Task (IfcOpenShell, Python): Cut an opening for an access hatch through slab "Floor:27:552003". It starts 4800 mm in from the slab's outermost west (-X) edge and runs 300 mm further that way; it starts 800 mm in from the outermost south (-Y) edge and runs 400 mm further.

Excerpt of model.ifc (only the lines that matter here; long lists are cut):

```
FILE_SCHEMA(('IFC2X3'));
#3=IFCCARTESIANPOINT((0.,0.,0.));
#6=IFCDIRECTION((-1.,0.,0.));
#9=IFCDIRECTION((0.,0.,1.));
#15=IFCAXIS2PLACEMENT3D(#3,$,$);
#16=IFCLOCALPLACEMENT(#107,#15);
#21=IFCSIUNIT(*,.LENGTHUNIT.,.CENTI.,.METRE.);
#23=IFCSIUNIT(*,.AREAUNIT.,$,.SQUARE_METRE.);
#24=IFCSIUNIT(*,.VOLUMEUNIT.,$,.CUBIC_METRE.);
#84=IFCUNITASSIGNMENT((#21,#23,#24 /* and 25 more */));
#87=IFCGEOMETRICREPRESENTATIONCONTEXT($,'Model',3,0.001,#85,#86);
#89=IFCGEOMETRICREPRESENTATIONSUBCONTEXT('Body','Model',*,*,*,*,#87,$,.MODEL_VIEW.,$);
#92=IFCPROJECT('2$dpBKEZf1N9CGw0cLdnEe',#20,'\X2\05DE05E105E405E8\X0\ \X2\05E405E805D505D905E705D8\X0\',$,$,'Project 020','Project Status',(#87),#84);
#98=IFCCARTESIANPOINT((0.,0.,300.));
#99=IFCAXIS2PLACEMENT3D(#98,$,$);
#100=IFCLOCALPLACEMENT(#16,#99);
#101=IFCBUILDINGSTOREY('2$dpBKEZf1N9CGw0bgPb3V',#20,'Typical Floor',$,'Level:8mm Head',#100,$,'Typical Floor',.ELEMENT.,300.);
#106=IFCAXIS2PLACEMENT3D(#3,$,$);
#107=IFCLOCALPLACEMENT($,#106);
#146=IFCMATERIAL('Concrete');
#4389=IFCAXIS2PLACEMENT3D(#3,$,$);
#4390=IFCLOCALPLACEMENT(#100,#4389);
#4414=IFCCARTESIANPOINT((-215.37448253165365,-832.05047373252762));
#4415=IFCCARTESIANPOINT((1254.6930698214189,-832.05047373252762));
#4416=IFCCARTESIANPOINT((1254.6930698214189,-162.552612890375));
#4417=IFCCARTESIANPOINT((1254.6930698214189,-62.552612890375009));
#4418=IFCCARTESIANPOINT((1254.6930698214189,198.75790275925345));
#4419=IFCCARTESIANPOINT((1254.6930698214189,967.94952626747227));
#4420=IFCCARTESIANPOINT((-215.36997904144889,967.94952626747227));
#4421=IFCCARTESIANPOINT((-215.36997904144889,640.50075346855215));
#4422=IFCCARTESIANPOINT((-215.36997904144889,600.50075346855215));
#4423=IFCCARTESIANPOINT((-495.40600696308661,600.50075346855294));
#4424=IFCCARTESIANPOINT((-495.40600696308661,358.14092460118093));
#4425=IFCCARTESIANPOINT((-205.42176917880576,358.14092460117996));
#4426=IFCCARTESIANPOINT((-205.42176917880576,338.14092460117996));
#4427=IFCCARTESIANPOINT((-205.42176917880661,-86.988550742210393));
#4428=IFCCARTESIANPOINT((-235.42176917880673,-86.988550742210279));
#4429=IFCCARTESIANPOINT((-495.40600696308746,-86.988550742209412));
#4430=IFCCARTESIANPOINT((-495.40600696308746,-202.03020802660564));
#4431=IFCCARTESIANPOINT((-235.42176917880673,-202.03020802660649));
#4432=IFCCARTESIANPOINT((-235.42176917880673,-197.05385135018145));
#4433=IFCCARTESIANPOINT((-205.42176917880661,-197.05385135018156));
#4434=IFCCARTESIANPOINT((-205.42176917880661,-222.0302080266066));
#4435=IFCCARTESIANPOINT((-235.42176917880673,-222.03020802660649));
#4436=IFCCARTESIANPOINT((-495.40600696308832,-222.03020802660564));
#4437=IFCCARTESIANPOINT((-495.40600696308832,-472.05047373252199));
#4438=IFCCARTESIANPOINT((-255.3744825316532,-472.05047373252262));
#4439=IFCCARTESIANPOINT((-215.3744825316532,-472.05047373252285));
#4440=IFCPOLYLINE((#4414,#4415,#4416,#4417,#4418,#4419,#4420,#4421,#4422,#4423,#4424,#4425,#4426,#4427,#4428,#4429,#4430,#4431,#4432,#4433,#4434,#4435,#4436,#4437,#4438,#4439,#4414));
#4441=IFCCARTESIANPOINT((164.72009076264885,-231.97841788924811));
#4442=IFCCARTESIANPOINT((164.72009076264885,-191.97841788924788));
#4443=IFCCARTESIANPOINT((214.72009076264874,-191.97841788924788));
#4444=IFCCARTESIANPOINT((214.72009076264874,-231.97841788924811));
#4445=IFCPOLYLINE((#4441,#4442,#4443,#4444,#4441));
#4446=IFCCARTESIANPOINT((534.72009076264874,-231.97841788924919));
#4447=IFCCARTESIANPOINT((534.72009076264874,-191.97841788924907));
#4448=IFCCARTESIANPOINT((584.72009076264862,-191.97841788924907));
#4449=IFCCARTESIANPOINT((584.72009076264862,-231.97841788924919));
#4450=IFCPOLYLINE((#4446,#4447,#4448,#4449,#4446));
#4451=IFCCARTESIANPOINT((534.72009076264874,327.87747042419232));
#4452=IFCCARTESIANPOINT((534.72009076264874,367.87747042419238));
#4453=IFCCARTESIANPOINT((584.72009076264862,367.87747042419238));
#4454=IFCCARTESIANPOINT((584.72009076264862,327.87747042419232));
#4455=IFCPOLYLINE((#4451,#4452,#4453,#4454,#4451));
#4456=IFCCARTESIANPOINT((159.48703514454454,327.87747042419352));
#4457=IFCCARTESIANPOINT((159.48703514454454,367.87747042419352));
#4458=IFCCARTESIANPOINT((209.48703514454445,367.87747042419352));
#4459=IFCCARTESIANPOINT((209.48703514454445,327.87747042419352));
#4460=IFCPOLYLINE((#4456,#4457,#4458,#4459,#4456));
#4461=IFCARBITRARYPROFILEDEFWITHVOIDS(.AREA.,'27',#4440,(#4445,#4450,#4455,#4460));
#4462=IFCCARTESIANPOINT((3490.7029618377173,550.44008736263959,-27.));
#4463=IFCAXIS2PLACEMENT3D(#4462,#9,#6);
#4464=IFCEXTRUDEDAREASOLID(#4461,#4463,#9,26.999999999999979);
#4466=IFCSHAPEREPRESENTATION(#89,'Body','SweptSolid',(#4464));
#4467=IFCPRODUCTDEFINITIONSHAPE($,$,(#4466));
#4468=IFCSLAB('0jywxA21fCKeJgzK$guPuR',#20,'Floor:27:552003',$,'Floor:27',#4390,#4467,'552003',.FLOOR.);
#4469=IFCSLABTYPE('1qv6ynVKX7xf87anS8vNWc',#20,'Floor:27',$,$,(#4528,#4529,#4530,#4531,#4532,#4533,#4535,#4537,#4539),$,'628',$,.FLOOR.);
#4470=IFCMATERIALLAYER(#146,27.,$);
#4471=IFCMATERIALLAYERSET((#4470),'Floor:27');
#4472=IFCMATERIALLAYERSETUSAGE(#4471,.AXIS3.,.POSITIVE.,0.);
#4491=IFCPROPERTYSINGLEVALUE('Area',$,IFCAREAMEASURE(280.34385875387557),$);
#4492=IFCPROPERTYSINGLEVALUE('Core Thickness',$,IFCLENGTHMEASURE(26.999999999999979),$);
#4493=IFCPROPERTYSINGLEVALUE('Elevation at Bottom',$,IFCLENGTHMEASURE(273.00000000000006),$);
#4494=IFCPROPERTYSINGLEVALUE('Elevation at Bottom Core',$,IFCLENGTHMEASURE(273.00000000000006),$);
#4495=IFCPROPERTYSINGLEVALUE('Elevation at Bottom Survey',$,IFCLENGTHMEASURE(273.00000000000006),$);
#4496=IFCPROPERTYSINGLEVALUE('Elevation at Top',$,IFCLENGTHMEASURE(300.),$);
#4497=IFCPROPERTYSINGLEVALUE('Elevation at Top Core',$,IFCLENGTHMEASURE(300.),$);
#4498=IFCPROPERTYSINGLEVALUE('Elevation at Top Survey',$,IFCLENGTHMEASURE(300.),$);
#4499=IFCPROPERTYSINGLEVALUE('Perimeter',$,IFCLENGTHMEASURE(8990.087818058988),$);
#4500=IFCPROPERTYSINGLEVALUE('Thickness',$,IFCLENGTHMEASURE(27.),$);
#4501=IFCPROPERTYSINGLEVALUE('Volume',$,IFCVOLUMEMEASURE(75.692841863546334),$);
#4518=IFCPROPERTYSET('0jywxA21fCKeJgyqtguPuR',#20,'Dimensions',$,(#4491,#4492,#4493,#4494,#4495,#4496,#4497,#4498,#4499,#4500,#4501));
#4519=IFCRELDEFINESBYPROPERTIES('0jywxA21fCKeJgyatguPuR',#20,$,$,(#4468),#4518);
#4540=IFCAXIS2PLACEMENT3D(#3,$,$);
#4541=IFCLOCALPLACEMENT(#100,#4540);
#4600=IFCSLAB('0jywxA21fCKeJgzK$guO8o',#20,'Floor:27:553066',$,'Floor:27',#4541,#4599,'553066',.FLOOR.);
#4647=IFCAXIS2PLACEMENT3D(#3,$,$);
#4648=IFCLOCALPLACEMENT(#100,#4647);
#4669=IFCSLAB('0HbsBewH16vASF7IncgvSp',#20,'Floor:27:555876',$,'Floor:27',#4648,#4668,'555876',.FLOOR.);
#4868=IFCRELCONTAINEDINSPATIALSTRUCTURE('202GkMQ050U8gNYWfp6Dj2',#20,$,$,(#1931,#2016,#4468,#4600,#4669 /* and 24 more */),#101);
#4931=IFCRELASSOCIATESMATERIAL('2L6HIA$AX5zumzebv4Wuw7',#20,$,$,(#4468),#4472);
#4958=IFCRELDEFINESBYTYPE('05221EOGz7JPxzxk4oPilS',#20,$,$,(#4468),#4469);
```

```python
import numpy as np
import ifcopenshell
import ifcopenshell.api.feature
import ifcopenshell.api.geometry
import ifcopenshell.api.pset
import ifcopenshell.api.root
import ifcopenshell.geom
import ifcopenshell.util.element
import ifcopenshell.util.placement
import ifcopenshell.util.representation
import ifcopenshell.util.shape
import ifcopenshell.util.unit

model = ifcopenshell.open("model.ifc")
unit_scale = ifcopenshell.util.unit.calculate_unit_scale(model)
area_scale = ifcopenshell.util.unit.calculate_unit_scale(model, "AREAUNIT")
volume_scale = ifcopenshell.util.unit.calculate_unit_scale(model, "VOLUMEUNIT")
settings = ifcopenshell.geom.settings()


def volume(element):
    """Net volume in cubic metres, openings subtracted."""
    shape = ifcopenshell.geom.create_shape(settings, element)
    return ifcopenshell.util.shape.get_volume(shape.geometry)


slab = model.by_guid("0jywxA21fCKeJgzK$guPuR")
before = volume(slab)

# Extent in the slab's own axes, in metres. The edges named are its -X and -Y sides.
slab_shape = ifcopenshell.geom.create_shape(settings, slab)
vertices = ifcopenshell.util.shape.get_vertices(slab_shape.geometry)
x_min, y_min, bottom = vertices.min(axis=0)
top = vertices[:, 2].max()

opening = ifcopenshell.api.root.create_entity(model, ifc_class="IfcOpeningElement", name="Access hatch opening")
context = ifcopenshell.util.representation.get_context(model, "Model", "Body", "MODEL_VIEW")
width, depth = 0.3, 0.4
outline = [(0.0, 0.0), (width, 0.0), (width, depth), (0.0, depth), (0.0, 0.0)]
# Overshoot both faces by 50 mm so the cut is clean.
shape = ifcopenshell.api.geometry.add_slab_representation(
    model, context=context, depth=top - bottom + 0.1, polyline=outline
)
ifcopenshell.api.geometry.assign_representation(model, product=opening, representation=shape)

matrix = ifcopenshell.util.placement.get_local_placement(slab.ObjectPlacement)
matrix[:, 3] = matrix @ np.append(np.array([x_min + 4.8, y_min + 0.8, bottom - 0.05]) / unit_scale, 1.0)
ifcopenshell.api.geometry.edit_object_placement(model, product=opening, matrix=matrix, is_si=False)
ifcopenshell.api.feature.add_feature(model, feature=opening, element=slab)

after = volume(slab)

# Update the slab's stored quantities.
pset = model.by_id(ifcopenshell.util.element.get_pset(slab, "Dimensions", should_inherit=False)["id"])
ifcopenshell.api.pset.edit_pset(model, pset=pset, properties={
    "Area": model.create_entity("IfcAreaMeasure", after / (top - bottom) / area_scale),
    "Volume": model.create_entity("IfcVolumeMeasure", after / volume_scale),
})

print(f"slab volume {before:.3f} -> {after:.3f} m3")

model.write("model-out.ifc")
```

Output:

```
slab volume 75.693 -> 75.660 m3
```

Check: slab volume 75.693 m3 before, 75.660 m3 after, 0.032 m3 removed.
